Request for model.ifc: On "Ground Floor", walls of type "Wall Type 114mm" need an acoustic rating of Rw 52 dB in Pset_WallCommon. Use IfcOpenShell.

First a look at what the model holds.

```python
import ifcopenshell
import ifcopenshell.util.element

model = ifcopenshell.open("model.ifc")
print(model.schema)
storey = next(s for s in model.by_type("IfcBuildingStorey") if s.Name == "Ground Floor")
walls = [e for e in ifcopenshell.util.element.get_decomposition(storey) if e.is_a("IfcWall")]
seen = {}
for e in walls:
    element_type = ifcopenshell.util.element.get_type(e)
    key = (element_type.Name if element_type != e and element_type else None, ifcopenshell.util.element.get_pset(e, "Pset_WallCommon", "AcousticRating"))
    seen[key] = seen.get(key, 0) + 1
for (name, value), count in sorted(seen.items(), key=str):
    print(count, "x", name, "|", value)
```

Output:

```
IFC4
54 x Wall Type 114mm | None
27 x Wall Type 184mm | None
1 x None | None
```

```python
import ifcopenshell
import ifcopenshell.api.pset
import ifcopenshell.util.element

model = ifcopenshell.open("model.ifc")

storey = next(s for s in model.by_type("IfcBuildingStorey") if s.Name == "Ground Floor")
walls = [e for e in ifcopenshell.util.element.get_decomposition(storey) if e.is_a("IfcWall")]

count = 0
for e in walls:
    element_type = ifcopenshell.util.element.get_type(e)
    if element_type in (None, e) or element_type.Name != "Wall Type 114mm":
        continue
    # add_pset returns the element's existing set when there is one.
    pset = ifcopenshell.api.pset.add_pset(model, product=e, name="Pset_WallCommon")
    ifcopenshell.api.pset.edit_pset(model, pset=pset, properties={"AcousticRating": "Rw 52 dB"})
    count += 1

print(count, "walls updated")

model.write("model-out.ifc")
```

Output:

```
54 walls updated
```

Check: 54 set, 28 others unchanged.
